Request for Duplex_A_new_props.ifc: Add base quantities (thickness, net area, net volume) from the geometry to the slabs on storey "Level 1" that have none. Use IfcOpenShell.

First a look at what the model holds.

```python
import ifcopenshell
import ifcopenshell.util.element
import ifcopenshell.util.unit

model = ifcopenshell.open("Duplex_A_new_props.ifc")
print(model.schema)
for unit_type in ("LENGTHUNIT", "AREAUNIT", "VOLUMEUNIT"):
    print(unit_type, ifcopenshell.util.unit.calculate_unit_scale(model, unit_type))
storey = next(s for s in model.by_type("IfcBuildingStorey") if s.Name == "Level 1")
slabs = [e for e in ifcopenshell.util.element.get_decomposition(storey) if e.is_a("IfcSlab")]
for e in sorted(slabs, key=lambda e: e.id()):
    print(e.id(), e.is_a(), e.Name, list(ifcopenshell.util.element.get_psets(e, qtos_only=True)), sep=" | ")
```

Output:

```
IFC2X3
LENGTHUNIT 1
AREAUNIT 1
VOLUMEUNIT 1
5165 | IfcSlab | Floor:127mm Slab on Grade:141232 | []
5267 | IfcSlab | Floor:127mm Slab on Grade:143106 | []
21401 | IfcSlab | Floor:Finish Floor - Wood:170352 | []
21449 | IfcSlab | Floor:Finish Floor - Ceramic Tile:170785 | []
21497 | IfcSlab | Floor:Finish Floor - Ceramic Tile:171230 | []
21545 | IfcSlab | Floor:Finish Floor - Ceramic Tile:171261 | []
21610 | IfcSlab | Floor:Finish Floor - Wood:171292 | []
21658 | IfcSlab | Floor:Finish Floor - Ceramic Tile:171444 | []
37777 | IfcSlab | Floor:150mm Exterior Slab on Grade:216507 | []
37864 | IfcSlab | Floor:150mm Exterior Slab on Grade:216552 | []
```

```python
import ifcopenshell
import ifcopenshell.api.pset
import ifcopenshell.geom
import ifcopenshell.util.element
import ifcopenshell.util.shape
import ifcopenshell.util.unit

model = ifcopenshell.open("Duplex_A_new_props.ifc")
unit_scale = ifcopenshell.util.unit.calculate_unit_scale(model)
area_scale = ifcopenshell.util.unit.calculate_unit_scale(model, "AREAUNIT")
volume_scale = ifcopenshell.util.unit.calculate_unit_scale(model, "VOLUMEUNIT")
settings = ifcopenshell.geom.settings()

storey = next(s for s in model.by_type("IfcBuildingStorey") if s.Name == "Level 1")
slabs = [e for e in ifcopenshell.util.element.get_decomposition(storey) if e.is_a("IfcSlab")]

for e in sorted(slabs, key=lambda e: e.id()):
    if ifcopenshell.util.element.get_psets(e, qtos_only=True, should_inherit=False):
        continue
    # Geometry comes back in metres, in the element's own axes.
    shape = ifcopenshell.geom.create_shape(settings, e)
    values = {
        "Width": ifcopenshell.util.shape.get_z(shape.geometry) / unit_scale,
        "NetArea": ifcopenshell.util.shape.get_footprint_area(shape.geometry) / area_scale,
        "NetVolume": ifcopenshell.util.shape.get_volume(shape.geometry) / volume_scale,
    }
    qto = ifcopenshell.api.pset.add_qto(model, product=e, name="BaseQuantities")
    ifcopenshell.api.pset.edit_qto(model, qto=qto, properties=values)
    print(e.id(), {k: round(v, 3) for k, v in values.items()})

model.write("Duplex_A_new_props_edited.ifc")
```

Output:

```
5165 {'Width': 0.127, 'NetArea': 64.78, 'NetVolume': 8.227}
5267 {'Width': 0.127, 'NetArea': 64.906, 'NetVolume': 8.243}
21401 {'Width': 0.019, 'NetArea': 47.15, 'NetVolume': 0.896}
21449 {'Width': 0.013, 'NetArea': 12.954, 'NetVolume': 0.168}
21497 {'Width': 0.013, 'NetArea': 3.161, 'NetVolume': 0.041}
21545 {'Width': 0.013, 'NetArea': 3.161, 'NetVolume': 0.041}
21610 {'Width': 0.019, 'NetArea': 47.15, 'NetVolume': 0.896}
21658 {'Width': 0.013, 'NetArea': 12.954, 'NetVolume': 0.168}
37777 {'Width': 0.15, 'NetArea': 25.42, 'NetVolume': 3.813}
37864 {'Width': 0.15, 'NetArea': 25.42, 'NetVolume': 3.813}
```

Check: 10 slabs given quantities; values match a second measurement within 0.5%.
